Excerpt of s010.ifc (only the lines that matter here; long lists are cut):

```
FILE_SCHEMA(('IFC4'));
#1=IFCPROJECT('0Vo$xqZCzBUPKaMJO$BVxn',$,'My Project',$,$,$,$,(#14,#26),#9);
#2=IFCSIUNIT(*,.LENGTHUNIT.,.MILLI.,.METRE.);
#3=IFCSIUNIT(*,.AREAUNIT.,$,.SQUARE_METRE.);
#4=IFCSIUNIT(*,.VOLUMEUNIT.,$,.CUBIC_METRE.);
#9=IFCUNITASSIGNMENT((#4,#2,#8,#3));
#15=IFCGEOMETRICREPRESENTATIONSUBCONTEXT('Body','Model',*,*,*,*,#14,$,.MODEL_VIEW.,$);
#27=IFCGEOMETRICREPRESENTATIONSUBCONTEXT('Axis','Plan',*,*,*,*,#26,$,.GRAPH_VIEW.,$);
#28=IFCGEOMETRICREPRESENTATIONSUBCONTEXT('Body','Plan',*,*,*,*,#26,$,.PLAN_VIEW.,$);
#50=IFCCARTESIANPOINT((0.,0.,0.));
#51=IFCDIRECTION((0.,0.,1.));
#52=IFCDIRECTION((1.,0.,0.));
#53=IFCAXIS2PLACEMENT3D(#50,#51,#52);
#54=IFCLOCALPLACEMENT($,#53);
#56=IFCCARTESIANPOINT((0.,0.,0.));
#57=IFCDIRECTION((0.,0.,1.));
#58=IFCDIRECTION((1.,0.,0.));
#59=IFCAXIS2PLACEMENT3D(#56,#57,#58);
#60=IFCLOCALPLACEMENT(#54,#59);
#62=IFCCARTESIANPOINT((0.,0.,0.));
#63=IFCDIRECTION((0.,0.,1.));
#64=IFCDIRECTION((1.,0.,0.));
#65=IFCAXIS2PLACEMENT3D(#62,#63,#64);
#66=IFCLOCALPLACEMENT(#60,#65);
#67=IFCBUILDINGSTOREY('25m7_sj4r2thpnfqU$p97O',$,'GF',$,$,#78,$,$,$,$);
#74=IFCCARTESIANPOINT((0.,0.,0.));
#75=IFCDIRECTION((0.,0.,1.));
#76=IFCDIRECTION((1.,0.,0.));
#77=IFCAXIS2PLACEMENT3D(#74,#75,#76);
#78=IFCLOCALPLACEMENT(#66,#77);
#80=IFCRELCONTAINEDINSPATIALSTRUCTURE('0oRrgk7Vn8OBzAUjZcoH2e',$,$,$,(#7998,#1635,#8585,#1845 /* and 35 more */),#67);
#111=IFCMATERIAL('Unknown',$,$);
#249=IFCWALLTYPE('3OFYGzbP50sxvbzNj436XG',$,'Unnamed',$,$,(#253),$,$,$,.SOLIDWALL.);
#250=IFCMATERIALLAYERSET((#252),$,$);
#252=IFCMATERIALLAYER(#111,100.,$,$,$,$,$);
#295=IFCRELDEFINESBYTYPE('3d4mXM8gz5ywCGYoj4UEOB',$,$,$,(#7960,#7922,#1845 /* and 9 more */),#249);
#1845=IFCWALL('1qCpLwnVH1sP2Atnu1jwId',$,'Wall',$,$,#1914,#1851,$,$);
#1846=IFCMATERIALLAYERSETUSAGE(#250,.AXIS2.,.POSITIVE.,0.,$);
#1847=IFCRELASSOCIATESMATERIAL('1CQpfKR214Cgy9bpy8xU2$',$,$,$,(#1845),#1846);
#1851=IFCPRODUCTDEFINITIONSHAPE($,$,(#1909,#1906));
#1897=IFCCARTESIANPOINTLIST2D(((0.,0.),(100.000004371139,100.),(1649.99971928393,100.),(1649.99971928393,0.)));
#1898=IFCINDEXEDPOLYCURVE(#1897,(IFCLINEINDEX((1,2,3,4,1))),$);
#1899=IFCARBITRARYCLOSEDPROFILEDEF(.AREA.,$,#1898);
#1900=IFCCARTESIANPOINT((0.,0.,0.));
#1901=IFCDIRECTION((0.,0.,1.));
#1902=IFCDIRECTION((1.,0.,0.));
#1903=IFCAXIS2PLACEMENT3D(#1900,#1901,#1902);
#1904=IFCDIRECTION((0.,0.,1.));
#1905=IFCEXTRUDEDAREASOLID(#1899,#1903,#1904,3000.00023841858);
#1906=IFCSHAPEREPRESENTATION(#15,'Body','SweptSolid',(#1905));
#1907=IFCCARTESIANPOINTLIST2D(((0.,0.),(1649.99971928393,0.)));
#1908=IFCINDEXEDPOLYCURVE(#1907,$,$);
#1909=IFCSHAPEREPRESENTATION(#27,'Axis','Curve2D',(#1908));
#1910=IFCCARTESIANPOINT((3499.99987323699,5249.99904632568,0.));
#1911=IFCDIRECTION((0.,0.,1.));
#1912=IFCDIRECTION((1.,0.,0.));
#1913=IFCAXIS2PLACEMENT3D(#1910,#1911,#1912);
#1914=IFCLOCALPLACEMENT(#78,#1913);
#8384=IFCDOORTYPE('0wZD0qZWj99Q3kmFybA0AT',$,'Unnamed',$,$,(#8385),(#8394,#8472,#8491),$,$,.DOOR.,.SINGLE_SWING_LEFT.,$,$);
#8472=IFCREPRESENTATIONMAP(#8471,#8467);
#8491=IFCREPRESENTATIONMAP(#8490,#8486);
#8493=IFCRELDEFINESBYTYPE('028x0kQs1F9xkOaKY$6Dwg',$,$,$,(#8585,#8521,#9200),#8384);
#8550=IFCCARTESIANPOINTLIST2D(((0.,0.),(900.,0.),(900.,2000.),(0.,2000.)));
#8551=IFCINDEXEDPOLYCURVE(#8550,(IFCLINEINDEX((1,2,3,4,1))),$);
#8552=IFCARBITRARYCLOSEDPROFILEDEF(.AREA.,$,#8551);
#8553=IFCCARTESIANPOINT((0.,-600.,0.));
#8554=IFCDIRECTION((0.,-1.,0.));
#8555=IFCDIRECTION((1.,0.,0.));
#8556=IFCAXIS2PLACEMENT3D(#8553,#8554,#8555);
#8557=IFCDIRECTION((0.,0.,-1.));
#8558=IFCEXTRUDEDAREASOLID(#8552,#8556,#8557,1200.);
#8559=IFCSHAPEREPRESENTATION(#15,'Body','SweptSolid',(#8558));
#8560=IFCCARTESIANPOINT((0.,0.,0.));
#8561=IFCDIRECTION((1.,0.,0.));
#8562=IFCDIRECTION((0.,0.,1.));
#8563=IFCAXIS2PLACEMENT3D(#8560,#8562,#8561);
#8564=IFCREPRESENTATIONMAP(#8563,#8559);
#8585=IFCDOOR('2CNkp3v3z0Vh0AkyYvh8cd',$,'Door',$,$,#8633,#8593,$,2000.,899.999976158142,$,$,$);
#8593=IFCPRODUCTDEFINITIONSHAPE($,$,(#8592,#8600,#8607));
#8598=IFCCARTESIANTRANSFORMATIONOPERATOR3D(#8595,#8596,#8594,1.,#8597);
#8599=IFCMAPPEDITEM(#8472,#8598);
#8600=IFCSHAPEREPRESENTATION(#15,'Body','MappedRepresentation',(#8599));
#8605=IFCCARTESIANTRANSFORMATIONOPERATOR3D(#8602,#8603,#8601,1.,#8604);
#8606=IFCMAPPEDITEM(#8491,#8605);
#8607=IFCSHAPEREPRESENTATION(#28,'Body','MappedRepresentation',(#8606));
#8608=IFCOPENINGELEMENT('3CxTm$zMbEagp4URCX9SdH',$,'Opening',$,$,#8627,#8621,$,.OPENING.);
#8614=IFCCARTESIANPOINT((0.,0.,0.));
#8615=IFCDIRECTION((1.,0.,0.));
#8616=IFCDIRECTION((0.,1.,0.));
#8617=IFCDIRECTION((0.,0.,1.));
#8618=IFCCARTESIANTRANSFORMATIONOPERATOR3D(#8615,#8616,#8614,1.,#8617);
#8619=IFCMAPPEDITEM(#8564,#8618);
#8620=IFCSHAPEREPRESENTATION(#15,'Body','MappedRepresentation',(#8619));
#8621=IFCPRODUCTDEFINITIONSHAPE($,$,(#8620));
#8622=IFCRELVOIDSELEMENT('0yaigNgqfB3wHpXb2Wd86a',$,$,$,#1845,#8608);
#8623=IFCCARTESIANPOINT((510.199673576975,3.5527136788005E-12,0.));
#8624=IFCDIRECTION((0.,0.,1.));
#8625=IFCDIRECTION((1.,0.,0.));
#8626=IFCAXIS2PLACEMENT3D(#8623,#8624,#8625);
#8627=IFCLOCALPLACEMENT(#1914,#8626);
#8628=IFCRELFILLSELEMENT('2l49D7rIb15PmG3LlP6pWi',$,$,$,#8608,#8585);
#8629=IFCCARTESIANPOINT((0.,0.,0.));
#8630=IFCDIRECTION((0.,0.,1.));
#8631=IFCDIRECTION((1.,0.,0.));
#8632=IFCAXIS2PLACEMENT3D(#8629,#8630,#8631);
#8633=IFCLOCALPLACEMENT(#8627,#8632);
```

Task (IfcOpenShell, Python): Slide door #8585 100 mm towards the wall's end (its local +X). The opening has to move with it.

```python
import ifcopenshell
import ifcopenshell.api.geometry
import ifcopenshell.util.placement
import ifcopenshell.util.unit

model = ifcopenshell.open("s010.ifc")
unit_scale = ifcopenshell.util.unit.calculate_unit_scale(model)

door = model.by_guid("2CNkp3v3z0Vh0AkyYvh8cd")
opening = door.FillsVoids[0].RelatingOpeningElement
wall = opening.VoidsElements[0].RelatingBuildingElement

wall_matrix = ifcopenshell.util.placement.get_local_placement(wall.ObjectPlacement)
shift = wall_matrix[:3, 0] * 0.1 / unit_scale
before = ifcopenshell.util.placement.get_local_placement(door.ObjectPlacement)[:3, 3].copy()

# The door is placed relative to its opening, so it follows when the opening moves.
matrix = ifcopenshell.util.placement.get_local_placement(opening.ObjectPlacement)
matrix[:3, 3] += shift
ifcopenshell.api.geometry.edit_object_placement(
    model, product=opening, matrix=matrix, is_si=False, should_transform_children=True
)

after = ifcopenshell.util.placement.get_local_placement(door.ObjectPlacement)[:3, 3]
print("door moved by", (after - before).round(3) + 0.0)

model.write("s010_rev.ifc")
```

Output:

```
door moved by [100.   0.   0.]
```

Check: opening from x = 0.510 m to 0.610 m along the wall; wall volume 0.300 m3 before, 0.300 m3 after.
